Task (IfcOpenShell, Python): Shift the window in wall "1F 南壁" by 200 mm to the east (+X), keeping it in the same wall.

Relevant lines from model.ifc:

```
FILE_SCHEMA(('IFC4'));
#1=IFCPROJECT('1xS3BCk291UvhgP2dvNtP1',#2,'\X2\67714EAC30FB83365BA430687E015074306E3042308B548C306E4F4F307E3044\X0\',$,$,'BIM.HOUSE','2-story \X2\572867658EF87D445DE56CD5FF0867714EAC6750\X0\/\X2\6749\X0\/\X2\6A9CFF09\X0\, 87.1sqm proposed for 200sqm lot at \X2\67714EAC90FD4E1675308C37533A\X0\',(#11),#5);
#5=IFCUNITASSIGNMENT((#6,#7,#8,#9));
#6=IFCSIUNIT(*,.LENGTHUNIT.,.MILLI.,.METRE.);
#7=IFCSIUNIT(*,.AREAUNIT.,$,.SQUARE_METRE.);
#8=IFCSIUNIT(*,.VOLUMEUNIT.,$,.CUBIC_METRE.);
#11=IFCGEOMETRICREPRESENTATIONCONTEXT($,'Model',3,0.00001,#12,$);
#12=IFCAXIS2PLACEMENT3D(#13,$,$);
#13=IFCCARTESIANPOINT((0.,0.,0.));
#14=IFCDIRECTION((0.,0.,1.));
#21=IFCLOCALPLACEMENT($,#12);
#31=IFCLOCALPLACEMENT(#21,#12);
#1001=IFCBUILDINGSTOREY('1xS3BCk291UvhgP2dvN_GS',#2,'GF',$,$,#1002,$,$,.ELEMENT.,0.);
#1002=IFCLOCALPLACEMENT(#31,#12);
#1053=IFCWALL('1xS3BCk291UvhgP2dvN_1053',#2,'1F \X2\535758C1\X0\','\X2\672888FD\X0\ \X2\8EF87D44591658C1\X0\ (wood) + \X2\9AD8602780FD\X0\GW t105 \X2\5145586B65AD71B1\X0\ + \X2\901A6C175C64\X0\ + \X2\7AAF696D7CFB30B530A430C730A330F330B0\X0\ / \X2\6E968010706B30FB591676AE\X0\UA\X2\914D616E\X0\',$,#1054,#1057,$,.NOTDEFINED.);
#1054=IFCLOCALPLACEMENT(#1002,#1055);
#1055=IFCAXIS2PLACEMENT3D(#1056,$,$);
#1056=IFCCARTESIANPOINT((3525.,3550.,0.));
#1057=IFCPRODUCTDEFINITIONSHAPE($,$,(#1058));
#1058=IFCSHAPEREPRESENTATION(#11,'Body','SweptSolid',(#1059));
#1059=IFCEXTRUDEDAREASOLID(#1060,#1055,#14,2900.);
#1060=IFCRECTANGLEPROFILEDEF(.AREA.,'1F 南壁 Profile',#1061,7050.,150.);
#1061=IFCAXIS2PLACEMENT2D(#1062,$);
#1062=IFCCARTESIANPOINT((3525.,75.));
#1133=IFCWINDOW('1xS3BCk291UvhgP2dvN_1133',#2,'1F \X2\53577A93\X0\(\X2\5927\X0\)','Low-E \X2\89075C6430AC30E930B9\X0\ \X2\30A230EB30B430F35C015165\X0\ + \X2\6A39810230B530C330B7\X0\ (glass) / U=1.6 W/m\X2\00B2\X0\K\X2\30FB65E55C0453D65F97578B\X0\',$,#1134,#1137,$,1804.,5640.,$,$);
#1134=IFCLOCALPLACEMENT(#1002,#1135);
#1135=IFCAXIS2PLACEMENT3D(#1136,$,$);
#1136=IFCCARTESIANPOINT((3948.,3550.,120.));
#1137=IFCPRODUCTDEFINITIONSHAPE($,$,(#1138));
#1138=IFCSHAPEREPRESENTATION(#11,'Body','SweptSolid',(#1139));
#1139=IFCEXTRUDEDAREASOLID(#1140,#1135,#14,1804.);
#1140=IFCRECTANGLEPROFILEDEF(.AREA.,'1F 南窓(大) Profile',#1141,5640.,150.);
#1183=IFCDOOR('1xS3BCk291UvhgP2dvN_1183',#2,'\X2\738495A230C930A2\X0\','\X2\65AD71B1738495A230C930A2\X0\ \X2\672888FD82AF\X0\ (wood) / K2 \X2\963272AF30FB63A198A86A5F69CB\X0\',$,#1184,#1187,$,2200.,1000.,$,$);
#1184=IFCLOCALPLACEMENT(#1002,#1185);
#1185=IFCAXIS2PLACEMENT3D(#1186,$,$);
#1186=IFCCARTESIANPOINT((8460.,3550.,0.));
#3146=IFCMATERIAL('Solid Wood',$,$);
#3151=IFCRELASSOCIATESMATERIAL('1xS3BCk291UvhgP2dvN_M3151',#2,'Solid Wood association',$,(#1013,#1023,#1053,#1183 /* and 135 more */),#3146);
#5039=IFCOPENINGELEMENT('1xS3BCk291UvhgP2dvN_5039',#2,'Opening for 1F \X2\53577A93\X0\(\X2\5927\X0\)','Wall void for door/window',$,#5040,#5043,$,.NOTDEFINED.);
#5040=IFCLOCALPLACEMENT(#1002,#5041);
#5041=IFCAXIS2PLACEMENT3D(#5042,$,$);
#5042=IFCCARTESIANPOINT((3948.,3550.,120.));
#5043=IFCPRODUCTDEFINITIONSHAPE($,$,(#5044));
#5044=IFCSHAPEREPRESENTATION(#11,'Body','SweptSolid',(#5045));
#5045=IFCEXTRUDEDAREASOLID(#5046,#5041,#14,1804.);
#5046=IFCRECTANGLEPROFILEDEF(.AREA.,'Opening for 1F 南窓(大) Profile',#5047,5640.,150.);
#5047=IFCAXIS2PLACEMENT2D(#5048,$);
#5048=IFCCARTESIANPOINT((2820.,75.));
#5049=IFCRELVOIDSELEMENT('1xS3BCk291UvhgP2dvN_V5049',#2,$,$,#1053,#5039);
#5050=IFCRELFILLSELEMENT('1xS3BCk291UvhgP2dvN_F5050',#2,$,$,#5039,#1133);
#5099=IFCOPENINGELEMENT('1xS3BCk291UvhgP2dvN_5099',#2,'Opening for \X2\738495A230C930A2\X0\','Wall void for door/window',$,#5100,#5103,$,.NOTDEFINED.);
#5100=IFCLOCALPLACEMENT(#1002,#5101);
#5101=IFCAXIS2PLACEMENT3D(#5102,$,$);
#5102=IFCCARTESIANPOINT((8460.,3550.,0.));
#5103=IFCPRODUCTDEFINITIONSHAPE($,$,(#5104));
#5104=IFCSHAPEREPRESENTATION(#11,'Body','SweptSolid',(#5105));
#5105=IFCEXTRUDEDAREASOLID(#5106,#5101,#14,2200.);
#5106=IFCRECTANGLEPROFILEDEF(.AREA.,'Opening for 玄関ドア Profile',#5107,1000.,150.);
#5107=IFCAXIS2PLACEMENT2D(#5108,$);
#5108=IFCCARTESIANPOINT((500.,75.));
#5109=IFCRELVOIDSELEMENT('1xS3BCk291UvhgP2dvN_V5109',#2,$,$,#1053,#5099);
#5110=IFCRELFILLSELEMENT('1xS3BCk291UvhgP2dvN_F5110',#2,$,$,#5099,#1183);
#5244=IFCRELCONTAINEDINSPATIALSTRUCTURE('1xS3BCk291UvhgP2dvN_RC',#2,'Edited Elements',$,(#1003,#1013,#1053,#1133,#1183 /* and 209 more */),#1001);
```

```python
import ifcopenshell
import ifcopenshell.api.geometry
import ifcopenshell.util.placement
import ifcopenshell.util.unit

model = ifcopenshell.open("model.ifc")
unit_scale = ifcopenshell.util.unit.calculate_unit_scale(model)

window = model.by_guid("1xS3BCk291UvhgP2dvN_1133")
opening = window.FillsVoids[0].RelatingOpeningElement
wall = opening.VoidsElements[0].RelatingBuildingElement

wall_matrix = ifcopenshell.util.placement.get_local_placement(wall.ObjectPlacement)
shift = wall_matrix[:3, 0] * 0.2 / unit_scale
before = ifcopenshell.util.placement.get_local_placement(window.ObjectPlacement)[:3, 3].copy()

# The window is not placed relative to its opening, so move both.
for product in (opening, window):
    matrix = ifcopenshell.util.placement.get_local_placement(product.ObjectPlacement)
    matrix[:3, 3] += shift
    ifcopenshell.api.geometry.edit_object_placement(model, product=product, matrix=matrix, is_si=False)

after = ifcopenshell.util.placement.get_local_placement(window.ObjectPlacement)[:3, 3]
print("window moved by", (after - before).round(3) + 0.0)

model.write("model_edited.ifc")
```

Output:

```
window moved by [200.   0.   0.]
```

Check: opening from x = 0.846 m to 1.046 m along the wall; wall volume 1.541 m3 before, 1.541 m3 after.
